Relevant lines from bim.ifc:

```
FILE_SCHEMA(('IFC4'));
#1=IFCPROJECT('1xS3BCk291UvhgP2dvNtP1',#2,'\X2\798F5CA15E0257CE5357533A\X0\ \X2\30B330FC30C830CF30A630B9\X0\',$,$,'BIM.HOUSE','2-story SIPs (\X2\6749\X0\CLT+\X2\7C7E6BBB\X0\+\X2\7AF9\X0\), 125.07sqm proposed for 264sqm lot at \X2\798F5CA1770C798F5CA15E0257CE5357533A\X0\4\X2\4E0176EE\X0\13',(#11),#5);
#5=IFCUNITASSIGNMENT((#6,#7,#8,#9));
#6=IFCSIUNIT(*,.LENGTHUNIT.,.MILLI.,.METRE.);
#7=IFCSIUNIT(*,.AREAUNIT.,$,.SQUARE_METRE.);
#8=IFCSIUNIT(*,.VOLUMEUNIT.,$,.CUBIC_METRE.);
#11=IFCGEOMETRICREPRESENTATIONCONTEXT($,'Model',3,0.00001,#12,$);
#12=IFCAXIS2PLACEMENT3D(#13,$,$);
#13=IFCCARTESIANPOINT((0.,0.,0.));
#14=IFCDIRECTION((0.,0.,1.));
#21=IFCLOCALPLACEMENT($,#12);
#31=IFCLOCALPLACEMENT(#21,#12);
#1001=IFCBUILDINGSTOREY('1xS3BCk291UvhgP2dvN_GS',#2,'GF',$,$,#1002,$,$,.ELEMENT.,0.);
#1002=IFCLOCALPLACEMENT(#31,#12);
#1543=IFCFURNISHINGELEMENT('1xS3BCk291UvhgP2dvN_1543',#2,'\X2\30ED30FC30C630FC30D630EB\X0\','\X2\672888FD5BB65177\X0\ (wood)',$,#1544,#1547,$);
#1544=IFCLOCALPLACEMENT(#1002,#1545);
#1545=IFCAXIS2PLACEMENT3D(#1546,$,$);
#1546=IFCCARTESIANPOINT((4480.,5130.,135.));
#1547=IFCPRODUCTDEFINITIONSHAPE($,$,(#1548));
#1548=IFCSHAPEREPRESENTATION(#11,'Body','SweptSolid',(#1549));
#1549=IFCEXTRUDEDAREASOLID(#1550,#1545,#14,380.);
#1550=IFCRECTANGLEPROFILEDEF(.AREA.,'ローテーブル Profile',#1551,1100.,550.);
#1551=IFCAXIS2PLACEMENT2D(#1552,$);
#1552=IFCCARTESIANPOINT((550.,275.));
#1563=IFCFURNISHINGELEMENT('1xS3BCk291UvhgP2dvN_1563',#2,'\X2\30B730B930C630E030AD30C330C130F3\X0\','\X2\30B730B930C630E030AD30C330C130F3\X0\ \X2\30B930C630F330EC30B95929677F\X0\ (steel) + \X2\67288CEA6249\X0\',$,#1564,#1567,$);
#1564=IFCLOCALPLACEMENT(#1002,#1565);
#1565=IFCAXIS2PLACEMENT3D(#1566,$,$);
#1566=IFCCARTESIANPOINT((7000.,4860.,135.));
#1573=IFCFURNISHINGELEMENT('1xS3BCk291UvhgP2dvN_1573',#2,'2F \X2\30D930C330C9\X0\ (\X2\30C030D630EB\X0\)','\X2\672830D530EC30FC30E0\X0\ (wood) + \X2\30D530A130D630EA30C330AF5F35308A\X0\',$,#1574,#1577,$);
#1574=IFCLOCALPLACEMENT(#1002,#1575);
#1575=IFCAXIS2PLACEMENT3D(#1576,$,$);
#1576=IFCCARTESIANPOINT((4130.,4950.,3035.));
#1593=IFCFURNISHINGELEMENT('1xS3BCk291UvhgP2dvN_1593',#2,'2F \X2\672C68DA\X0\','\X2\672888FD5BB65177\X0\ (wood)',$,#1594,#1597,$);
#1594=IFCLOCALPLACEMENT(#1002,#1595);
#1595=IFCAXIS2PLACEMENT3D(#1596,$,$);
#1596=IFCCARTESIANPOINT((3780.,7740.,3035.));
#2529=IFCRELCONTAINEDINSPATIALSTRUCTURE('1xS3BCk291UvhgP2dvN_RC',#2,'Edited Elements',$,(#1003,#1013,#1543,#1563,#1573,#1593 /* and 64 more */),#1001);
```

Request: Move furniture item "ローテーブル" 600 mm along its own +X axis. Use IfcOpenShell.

```python
import ifcopenshell
import ifcopenshell.api.geometry
import ifcopenshell.util.placement
import ifcopenshell.util.unit

model = ifcopenshell.open("bim.ifc")
unit_scale = ifcopenshell.util.unit.calculate_unit_scale(model)

item = model.by_id(1543)
matrix = ifcopenshell.util.placement.get_local_placement(item.ObjectPlacement)
matrix[:3, 3] += matrix[:3, 0] * 0.6 / unit_scale
ifcopenshell.api.geometry.edit_object_placement(model, product=item, matrix=matrix, is_si=False)

print(ifcopenshell.util.placement.get_local_placement(item.ObjectPlacement).round(3) + 0.0)

model.write("bim_rev.ifc")
```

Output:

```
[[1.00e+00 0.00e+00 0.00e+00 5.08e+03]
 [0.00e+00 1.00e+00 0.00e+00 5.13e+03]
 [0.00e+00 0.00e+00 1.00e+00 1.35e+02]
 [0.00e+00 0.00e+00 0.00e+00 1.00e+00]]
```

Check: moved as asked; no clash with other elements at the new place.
